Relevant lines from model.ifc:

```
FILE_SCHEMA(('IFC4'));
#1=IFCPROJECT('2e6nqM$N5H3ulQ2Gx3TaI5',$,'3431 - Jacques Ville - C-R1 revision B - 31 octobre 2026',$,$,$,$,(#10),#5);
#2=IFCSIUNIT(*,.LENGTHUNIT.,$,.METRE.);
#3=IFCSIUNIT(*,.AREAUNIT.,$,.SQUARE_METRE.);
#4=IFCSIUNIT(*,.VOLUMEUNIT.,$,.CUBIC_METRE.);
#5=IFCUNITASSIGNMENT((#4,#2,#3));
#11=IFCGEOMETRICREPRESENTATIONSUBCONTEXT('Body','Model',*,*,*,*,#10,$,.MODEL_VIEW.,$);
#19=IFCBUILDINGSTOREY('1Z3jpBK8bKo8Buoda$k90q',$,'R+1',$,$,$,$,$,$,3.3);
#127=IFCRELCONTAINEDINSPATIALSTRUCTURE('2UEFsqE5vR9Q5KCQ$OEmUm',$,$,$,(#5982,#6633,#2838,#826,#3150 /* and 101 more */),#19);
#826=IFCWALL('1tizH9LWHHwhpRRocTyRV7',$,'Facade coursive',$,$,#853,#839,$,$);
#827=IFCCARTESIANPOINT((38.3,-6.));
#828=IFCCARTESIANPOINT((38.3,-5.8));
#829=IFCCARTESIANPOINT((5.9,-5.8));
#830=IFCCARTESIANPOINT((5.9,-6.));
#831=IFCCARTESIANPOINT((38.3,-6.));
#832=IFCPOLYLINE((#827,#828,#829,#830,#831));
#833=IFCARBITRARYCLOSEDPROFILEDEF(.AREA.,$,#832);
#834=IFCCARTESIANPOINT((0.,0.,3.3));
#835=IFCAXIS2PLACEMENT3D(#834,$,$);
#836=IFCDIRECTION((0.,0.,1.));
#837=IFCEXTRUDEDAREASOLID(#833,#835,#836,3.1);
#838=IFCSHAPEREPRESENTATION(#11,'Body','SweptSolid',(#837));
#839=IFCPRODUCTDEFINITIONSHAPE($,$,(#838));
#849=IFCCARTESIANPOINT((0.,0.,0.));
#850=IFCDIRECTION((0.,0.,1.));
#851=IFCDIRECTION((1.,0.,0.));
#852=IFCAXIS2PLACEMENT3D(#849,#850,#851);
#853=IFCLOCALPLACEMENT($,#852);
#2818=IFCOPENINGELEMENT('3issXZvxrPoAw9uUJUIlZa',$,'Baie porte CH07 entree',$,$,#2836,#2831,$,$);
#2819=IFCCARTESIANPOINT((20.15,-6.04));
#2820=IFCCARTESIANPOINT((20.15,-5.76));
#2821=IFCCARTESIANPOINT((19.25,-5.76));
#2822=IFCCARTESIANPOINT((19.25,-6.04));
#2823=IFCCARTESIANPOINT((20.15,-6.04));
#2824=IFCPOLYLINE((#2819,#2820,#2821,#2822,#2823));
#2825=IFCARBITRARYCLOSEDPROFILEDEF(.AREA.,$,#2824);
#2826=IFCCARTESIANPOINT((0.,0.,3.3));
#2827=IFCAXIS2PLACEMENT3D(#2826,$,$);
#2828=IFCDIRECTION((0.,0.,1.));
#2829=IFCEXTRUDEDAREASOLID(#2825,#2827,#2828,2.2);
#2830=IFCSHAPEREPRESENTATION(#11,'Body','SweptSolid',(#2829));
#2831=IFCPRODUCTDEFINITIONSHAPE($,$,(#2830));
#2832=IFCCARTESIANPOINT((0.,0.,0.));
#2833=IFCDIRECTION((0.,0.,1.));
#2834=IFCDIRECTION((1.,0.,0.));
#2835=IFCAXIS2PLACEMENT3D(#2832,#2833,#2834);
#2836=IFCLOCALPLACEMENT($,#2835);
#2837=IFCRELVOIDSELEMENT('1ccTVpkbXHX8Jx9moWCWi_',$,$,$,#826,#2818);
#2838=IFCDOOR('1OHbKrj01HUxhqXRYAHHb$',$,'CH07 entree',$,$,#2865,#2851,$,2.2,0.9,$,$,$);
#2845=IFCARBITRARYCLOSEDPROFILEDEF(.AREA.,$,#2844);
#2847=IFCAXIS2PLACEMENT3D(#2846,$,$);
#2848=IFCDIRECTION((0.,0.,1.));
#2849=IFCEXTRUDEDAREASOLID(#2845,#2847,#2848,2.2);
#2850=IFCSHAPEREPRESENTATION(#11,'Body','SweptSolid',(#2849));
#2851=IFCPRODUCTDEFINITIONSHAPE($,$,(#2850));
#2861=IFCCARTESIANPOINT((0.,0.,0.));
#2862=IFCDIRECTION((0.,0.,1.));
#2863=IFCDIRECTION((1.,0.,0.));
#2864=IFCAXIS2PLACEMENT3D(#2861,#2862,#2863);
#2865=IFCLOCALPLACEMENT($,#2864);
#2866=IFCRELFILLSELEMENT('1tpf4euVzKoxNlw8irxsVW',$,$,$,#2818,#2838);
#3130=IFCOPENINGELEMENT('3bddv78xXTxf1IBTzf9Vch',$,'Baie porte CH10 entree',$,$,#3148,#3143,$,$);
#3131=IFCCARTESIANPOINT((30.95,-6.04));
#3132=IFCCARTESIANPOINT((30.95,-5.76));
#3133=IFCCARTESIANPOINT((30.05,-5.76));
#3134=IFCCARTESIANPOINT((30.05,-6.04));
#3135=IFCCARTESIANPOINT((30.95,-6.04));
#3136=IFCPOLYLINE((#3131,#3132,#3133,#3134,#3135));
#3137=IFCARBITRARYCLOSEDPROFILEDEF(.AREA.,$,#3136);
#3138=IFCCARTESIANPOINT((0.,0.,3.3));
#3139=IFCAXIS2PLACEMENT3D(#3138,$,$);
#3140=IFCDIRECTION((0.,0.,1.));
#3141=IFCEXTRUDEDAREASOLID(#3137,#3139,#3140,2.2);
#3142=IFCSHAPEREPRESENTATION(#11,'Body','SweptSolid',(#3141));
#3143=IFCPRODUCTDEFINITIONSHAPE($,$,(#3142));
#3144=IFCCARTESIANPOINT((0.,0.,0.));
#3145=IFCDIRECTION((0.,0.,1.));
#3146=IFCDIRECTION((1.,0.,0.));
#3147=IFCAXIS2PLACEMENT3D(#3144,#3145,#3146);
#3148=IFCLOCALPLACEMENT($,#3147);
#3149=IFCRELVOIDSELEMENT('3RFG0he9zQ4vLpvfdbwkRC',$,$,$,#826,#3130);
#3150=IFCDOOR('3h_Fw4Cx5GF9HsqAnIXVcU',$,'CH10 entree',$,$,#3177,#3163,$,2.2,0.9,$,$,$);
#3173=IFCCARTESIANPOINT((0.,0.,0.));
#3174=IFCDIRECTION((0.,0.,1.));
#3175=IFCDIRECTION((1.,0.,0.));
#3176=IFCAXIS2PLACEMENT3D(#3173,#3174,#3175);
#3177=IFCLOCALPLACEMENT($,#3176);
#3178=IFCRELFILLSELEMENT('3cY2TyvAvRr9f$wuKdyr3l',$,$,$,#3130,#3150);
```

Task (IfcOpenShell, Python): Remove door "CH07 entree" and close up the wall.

```python
import ifcopenshell
import ifcopenshell.api.feature
import ifcopenshell.api.root
import ifcopenshell.geom
import ifcopenshell.util.shape

model = ifcopenshell.open("model.ifc")
settings = ifcopenshell.geom.settings()


def volume(element):
    """Net volume in cubic metres, openings subtracted."""
    shape = ifcopenshell.geom.create_shape(settings, element)
    return ifcopenshell.util.shape.get_volume(shape.geometry)


door = model.by_guid("1OHbKrj01HUxhqXRYAHHb$")
opening = door.FillsVoids[0].RelatingOpeningElement
wall = opening.VoidsElements[0].RelatingBuildingElement
before = volume(wall)

ifcopenshell.api.root.remove_product(model, product=door)
ifcopenshell.api.feature.remove_feature(model, feature=opening)

after = volume(wall)

print(f"wall volume {before:.3f} -> {after:.3f} m3")

model.write("model_v2.ifc")
```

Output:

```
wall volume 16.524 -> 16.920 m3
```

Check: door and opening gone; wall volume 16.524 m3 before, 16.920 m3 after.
